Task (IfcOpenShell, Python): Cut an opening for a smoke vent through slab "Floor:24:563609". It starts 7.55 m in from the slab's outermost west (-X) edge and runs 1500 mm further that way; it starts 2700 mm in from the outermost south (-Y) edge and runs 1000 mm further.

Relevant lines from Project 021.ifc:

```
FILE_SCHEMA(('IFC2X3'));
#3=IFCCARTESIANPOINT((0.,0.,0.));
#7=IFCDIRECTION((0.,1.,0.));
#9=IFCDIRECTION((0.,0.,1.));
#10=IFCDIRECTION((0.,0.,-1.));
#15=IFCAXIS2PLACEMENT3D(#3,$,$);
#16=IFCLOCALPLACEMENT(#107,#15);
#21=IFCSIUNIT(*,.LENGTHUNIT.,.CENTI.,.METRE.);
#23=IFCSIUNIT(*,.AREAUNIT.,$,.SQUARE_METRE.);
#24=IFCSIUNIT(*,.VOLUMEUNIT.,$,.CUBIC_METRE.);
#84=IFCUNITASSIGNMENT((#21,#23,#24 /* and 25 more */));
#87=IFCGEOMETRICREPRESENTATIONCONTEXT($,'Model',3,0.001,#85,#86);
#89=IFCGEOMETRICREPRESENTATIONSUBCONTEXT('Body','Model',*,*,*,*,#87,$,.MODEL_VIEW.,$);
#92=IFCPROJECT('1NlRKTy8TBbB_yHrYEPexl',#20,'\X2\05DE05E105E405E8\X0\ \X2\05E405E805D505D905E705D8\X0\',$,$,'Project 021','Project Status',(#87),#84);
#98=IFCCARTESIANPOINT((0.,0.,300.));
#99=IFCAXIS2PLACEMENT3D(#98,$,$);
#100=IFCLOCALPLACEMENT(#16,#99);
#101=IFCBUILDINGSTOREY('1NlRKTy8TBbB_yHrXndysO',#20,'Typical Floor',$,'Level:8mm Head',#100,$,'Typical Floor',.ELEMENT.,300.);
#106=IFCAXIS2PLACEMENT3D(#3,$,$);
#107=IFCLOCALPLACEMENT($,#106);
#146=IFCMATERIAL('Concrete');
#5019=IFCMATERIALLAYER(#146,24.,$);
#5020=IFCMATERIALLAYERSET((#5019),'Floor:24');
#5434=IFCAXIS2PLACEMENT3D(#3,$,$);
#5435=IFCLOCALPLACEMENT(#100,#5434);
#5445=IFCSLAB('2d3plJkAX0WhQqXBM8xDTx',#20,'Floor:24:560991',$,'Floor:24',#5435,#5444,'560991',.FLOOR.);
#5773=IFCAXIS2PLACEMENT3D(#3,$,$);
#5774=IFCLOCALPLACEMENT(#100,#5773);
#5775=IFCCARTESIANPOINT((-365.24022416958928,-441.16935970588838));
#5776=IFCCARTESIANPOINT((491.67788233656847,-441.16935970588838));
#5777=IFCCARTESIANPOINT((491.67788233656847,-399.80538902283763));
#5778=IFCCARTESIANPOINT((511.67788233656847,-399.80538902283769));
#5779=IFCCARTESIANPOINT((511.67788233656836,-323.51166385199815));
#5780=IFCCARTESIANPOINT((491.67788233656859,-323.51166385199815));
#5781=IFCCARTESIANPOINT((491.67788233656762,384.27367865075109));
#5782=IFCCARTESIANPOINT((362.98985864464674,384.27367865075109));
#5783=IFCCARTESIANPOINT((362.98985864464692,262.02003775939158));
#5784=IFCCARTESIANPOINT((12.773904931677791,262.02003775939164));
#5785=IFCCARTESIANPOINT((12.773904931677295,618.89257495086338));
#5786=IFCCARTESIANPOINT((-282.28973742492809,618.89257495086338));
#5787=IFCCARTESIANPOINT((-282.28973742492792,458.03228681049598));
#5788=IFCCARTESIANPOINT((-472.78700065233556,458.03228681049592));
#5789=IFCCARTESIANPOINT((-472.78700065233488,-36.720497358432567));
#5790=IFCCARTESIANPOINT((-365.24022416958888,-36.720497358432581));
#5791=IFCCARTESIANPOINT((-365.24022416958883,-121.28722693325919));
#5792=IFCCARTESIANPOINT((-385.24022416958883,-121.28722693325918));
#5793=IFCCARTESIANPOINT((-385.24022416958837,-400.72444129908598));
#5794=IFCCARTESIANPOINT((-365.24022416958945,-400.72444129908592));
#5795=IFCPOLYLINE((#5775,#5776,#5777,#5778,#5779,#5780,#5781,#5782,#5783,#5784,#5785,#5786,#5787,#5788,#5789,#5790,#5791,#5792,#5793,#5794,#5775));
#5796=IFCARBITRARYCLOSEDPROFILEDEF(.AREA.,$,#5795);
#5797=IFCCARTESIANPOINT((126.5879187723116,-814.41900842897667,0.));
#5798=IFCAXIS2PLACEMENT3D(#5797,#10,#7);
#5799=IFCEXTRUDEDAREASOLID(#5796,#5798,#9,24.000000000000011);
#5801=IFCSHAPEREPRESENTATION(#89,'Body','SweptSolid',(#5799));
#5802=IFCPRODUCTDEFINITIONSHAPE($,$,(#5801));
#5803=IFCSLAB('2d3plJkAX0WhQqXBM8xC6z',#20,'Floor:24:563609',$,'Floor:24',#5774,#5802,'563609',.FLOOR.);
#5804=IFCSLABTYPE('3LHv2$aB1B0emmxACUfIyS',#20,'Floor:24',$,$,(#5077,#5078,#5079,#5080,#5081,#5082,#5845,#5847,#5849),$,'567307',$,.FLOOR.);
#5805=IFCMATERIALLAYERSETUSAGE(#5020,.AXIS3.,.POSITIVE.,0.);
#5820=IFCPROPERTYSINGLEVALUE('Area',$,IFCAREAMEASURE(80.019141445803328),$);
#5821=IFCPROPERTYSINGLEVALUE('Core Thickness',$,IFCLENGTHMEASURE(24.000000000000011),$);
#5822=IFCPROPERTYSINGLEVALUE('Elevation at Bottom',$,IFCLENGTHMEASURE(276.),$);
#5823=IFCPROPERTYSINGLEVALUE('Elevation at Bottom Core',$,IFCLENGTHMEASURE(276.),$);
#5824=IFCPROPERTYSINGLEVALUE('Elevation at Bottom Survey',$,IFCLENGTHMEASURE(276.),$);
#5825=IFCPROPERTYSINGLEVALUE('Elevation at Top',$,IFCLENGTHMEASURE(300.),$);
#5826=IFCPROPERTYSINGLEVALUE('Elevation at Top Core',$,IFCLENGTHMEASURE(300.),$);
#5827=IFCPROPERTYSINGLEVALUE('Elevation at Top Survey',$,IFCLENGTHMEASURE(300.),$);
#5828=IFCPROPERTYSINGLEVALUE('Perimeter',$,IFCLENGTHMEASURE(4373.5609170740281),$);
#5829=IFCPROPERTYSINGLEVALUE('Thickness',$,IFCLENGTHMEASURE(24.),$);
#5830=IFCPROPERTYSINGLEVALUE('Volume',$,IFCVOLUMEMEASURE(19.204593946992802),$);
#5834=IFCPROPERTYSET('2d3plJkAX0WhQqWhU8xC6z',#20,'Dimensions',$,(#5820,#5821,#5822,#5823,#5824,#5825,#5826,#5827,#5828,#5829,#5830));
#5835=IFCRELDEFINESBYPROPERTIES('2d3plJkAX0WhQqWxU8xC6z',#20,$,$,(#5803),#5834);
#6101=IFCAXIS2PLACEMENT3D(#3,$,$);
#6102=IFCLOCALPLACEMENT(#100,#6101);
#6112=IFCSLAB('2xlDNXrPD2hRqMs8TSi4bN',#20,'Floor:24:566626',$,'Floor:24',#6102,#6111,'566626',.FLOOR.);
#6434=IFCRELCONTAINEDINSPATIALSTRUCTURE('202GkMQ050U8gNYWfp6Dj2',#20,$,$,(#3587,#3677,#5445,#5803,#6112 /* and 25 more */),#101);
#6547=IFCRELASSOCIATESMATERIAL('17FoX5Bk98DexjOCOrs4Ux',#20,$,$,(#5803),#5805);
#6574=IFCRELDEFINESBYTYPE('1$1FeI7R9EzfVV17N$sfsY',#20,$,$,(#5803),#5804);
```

```python
import numpy as np
import ifcopenshell
import ifcopenshell.api.feature
import ifcopenshell.api.geometry
import ifcopenshell.api.pset
import ifcopenshell.api.root
import ifcopenshell.geom
import ifcopenshell.util.element
import ifcopenshell.util.placement
import ifcopenshell.util.representation
import ifcopenshell.util.shape
import ifcopenshell.util.unit

model = ifcopenshell.open("Project 021.ifc")
unit_scale = ifcopenshell.util.unit.calculate_unit_scale(model)
area_scale = ifcopenshell.util.unit.calculate_unit_scale(model, "AREAUNIT")
volume_scale = ifcopenshell.util.unit.calculate_unit_scale(model, "VOLUMEUNIT")
settings = ifcopenshell.geom.settings()


def volume(element):
    """Net volume in cubic metres, openings subtracted."""
    shape = ifcopenshell.geom.create_shape(settings, element)
    return ifcopenshell.util.shape.get_volume(shape.geometry)


slab = model.by_guid("2d3plJkAX0WhQqXBM8xC6z")
before = volume(slab)

# Extent in the slab's own axes, in metres. The edges named are its -X and -Y sides.
slab_shape = ifcopenshell.geom.create_shape(settings, slab)
vertices = ifcopenshell.util.shape.get_vertices(slab_shape.geometry)
x_min, y_min, bottom = vertices.min(axis=0)
top = vertices[:, 2].max()

opening = ifcopenshell.api.root.create_entity(model, ifc_class="IfcOpeningElement", name="Smoke vent opening")
context = ifcopenshell.util.representation.get_context(model, "Model", "Body", "MODEL_VIEW")
width, depth = 1.5, 1
outline = [(0.0, 0.0), (width, 0.0), (width, depth), (0.0, depth), (0.0, 0.0)]
# Overshoot both faces by 50 mm so the cut is clean.
shape = ifcopenshell.api.geometry.add_slab_representation(
    model, context=context, depth=top - bottom + 0.1, polyline=outline
)
ifcopenshell.api.geometry.assign_representation(model, product=opening, representation=shape)

matrix = ifcopenshell.util.placement.get_local_placement(slab.ObjectPlacement)
matrix[:, 3] = matrix @ np.append(np.array([x_min + 7.55, y_min + 2.7, bottom - 0.05]) / unit_scale, 1.0)
ifcopenshell.api.geometry.edit_object_placement(model, product=opening, matrix=matrix, is_si=False)
ifcopenshell.api.feature.add_feature(model, feature=opening, element=slab)

after = volume(slab)

# Update the slab's stored quantities.
pset = model.by_id(ifcopenshell.util.element.get_pset(slab, "Dimensions", should_inherit=False)["id"])
ifcopenshell.api.pset.edit_pset(model, pset=pset, properties={
    "Area": model.create_entity("IfcAreaMeasure", after / (top - bottom) / area_scale),
    "Volume": model.create_entity("IfcVolumeMeasure", after / volume_scale),
})

print(f"slab volume {before:.3f} -> {after:.3f} m3")

model.write("Project 021_v2.ifc")
```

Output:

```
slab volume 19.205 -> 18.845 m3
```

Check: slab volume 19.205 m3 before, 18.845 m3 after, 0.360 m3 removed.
